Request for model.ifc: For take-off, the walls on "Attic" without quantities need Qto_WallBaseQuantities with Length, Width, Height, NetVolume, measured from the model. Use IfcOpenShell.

First a look at what the model holds.

```python
import ifcopenshell
import ifcopenshell.util.element
import ifcopenshell.util.unit

model = ifcopenshell.open("model.ifc")
print(model.schema)
for unit_type in ("LENGTHUNIT", "AREAUNIT", "VOLUMEUNIT"):
    print(unit_type, ifcopenshell.util.unit.calculate_unit_scale(model, unit_type))
storey = next(s for s in model.by_type("IfcBuildingStorey") if s.Name == "Attic")
walls = [e for e in ifcopenshell.util.element.get_decomposition(storey) if e.is_a("IfcWall")]
for e in sorted(walls, key=lambda e: e.id()):
    print(e.id(), e.is_a(), e.Name, list(ifcopenshell.util.element.get_psets(e, qtos_only=True)), sep=" | ")
```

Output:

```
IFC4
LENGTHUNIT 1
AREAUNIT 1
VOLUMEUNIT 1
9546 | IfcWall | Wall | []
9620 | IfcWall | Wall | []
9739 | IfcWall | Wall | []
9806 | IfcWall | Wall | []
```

```python
import ifcopenshell
import ifcopenshell.api.pset
import ifcopenshell.geom
import ifcopenshell.util.element
import ifcopenshell.util.shape
import ifcopenshell.util.unit

model = ifcopenshell.open("model.ifc")
unit_scale = ifcopenshell.util.unit.calculate_unit_scale(model)
volume_scale = ifcopenshell.util.unit.calculate_unit_scale(model, "VOLUMEUNIT")
settings = ifcopenshell.geom.settings()

storey = next(s for s in model.by_type("IfcBuildingStorey") if s.Name == "Attic")
walls = [e for e in ifcopenshell.util.element.get_decomposition(storey) if e.is_a("IfcWall")]

for e in sorted(walls, key=lambda e: e.id()):
    if ifcopenshell.util.element.get_psets(e, qtos_only=True, should_inherit=False):
        continue
    # Geometry comes back in metres, in the element's own axes.
    shape = ifcopenshell.geom.create_shape(settings, e)
    values = {
        "Length": ifcopenshell.util.shape.get_x(shape.geometry) / unit_scale,
        "Width": ifcopenshell.util.shape.get_y(shape.geometry) / unit_scale,
        "Height": ifcopenshell.util.shape.get_z(shape.geometry) / unit_scale,
        "NetVolume": ifcopenshell.util.shape.get_volume(shape.geometry) / volume_scale,
    }
    qto = ifcopenshell.api.pset.add_qto(model, product=e, name="Qto_WallBaseQuantities")
    ifcopenshell.api.pset.edit_qto(model, qto=qto, properties=values)
    print(e.id(), {k: round(v, 3) for k, v in values.items()})

model.write("model_v2.ifc")
```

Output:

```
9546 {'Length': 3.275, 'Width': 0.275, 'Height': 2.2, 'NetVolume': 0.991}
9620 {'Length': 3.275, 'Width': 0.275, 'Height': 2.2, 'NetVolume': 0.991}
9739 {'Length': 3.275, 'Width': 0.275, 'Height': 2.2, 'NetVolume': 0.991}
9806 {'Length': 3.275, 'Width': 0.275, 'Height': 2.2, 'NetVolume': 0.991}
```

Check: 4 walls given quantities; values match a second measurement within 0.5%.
